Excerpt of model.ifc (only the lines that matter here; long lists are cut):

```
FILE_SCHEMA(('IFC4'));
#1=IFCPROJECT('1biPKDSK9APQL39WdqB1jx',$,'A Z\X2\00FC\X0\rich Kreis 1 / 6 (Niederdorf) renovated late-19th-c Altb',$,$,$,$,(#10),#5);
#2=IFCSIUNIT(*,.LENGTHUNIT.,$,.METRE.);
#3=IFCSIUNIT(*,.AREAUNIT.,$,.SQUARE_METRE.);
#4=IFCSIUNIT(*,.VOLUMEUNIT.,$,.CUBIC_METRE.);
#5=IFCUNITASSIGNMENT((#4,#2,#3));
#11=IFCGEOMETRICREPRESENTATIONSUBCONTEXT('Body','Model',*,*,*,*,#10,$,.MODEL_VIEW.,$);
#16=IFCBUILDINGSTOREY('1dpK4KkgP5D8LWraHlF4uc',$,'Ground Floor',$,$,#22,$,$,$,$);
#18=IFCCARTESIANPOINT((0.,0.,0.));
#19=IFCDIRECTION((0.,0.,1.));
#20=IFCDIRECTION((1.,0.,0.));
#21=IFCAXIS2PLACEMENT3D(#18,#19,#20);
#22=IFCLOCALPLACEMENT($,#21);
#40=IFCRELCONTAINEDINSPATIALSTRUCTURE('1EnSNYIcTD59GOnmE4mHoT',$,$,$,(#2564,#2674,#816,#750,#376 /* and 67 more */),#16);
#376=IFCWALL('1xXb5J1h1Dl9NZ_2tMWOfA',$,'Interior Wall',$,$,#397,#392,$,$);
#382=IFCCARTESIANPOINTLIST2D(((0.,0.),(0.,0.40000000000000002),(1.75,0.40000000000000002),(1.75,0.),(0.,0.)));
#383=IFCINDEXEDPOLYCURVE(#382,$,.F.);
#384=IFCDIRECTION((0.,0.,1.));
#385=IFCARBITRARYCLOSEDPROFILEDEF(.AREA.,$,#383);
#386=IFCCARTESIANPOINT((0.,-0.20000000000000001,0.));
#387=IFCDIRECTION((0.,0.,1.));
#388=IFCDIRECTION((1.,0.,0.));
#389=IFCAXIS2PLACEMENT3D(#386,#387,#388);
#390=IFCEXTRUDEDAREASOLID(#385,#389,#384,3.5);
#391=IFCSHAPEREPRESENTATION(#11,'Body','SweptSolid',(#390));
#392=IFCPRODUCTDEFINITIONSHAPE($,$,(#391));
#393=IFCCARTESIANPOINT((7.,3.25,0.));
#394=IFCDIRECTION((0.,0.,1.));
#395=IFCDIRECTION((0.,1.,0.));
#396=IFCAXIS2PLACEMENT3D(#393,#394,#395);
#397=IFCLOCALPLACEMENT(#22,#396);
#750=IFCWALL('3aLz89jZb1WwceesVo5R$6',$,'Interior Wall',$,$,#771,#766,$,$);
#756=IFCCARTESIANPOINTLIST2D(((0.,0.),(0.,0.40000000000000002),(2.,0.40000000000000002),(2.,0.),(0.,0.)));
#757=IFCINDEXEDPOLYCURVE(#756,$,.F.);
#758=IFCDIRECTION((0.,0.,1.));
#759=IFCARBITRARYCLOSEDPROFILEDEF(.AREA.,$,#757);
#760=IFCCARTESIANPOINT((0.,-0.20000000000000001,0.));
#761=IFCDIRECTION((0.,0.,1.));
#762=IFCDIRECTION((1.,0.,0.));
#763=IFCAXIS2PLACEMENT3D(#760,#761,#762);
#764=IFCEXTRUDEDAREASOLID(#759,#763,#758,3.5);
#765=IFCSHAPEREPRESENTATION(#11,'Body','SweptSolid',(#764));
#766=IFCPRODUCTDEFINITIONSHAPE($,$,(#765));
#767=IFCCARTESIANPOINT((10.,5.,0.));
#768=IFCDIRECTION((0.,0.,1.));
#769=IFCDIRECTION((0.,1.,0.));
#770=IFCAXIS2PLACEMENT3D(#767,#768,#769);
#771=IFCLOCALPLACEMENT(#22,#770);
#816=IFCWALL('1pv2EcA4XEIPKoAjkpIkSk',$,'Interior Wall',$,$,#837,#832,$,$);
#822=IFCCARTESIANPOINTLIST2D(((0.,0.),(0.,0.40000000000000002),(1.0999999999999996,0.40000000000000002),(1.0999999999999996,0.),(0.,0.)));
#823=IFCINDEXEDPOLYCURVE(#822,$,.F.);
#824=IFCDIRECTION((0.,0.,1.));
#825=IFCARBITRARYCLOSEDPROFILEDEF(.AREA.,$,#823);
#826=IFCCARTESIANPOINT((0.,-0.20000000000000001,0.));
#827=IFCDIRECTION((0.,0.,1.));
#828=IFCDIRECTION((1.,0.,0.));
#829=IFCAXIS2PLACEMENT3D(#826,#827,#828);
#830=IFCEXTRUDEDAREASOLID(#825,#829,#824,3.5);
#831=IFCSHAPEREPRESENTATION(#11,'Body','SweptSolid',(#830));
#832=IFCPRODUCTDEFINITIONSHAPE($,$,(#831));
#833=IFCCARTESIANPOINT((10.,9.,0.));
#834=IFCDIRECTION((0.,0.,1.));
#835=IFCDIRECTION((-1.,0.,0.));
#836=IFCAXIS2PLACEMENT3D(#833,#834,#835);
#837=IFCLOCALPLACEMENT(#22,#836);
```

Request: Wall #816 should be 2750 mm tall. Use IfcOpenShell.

```python
import ifcopenshell
import ifcopenshell.geom
import ifcopenshell.util.representation
import ifcopenshell.util.shape

model = ifcopenshell.open("model.ifc")
settings = ifcopenshell.geom.settings()


def volume(element):
    """Net volume in cubic metres, openings subtracted."""
    shape = ifcopenshell.geom.create_shape(settings, element)
    return ifcopenshell.util.shape.get_volume(shape.geometry)


wall = model.by_guid("1pv2EcA4XEIPKoAjkpIkSk")
before = volume(wall)

body = ifcopenshell.util.representation.get_representation(wall, "Model", "Body")
solid = body.Items[0]
old_height = solid.Depth
solid.Depth = 2.75
after = volume(wall)

print(f"height {old_height:g} -> {solid.Depth:g}, volume {before:.3f} -> {after:.3f} m3")

model.write("model_edited.ifc")
```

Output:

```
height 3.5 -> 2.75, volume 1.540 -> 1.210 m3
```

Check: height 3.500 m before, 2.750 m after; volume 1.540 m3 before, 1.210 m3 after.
